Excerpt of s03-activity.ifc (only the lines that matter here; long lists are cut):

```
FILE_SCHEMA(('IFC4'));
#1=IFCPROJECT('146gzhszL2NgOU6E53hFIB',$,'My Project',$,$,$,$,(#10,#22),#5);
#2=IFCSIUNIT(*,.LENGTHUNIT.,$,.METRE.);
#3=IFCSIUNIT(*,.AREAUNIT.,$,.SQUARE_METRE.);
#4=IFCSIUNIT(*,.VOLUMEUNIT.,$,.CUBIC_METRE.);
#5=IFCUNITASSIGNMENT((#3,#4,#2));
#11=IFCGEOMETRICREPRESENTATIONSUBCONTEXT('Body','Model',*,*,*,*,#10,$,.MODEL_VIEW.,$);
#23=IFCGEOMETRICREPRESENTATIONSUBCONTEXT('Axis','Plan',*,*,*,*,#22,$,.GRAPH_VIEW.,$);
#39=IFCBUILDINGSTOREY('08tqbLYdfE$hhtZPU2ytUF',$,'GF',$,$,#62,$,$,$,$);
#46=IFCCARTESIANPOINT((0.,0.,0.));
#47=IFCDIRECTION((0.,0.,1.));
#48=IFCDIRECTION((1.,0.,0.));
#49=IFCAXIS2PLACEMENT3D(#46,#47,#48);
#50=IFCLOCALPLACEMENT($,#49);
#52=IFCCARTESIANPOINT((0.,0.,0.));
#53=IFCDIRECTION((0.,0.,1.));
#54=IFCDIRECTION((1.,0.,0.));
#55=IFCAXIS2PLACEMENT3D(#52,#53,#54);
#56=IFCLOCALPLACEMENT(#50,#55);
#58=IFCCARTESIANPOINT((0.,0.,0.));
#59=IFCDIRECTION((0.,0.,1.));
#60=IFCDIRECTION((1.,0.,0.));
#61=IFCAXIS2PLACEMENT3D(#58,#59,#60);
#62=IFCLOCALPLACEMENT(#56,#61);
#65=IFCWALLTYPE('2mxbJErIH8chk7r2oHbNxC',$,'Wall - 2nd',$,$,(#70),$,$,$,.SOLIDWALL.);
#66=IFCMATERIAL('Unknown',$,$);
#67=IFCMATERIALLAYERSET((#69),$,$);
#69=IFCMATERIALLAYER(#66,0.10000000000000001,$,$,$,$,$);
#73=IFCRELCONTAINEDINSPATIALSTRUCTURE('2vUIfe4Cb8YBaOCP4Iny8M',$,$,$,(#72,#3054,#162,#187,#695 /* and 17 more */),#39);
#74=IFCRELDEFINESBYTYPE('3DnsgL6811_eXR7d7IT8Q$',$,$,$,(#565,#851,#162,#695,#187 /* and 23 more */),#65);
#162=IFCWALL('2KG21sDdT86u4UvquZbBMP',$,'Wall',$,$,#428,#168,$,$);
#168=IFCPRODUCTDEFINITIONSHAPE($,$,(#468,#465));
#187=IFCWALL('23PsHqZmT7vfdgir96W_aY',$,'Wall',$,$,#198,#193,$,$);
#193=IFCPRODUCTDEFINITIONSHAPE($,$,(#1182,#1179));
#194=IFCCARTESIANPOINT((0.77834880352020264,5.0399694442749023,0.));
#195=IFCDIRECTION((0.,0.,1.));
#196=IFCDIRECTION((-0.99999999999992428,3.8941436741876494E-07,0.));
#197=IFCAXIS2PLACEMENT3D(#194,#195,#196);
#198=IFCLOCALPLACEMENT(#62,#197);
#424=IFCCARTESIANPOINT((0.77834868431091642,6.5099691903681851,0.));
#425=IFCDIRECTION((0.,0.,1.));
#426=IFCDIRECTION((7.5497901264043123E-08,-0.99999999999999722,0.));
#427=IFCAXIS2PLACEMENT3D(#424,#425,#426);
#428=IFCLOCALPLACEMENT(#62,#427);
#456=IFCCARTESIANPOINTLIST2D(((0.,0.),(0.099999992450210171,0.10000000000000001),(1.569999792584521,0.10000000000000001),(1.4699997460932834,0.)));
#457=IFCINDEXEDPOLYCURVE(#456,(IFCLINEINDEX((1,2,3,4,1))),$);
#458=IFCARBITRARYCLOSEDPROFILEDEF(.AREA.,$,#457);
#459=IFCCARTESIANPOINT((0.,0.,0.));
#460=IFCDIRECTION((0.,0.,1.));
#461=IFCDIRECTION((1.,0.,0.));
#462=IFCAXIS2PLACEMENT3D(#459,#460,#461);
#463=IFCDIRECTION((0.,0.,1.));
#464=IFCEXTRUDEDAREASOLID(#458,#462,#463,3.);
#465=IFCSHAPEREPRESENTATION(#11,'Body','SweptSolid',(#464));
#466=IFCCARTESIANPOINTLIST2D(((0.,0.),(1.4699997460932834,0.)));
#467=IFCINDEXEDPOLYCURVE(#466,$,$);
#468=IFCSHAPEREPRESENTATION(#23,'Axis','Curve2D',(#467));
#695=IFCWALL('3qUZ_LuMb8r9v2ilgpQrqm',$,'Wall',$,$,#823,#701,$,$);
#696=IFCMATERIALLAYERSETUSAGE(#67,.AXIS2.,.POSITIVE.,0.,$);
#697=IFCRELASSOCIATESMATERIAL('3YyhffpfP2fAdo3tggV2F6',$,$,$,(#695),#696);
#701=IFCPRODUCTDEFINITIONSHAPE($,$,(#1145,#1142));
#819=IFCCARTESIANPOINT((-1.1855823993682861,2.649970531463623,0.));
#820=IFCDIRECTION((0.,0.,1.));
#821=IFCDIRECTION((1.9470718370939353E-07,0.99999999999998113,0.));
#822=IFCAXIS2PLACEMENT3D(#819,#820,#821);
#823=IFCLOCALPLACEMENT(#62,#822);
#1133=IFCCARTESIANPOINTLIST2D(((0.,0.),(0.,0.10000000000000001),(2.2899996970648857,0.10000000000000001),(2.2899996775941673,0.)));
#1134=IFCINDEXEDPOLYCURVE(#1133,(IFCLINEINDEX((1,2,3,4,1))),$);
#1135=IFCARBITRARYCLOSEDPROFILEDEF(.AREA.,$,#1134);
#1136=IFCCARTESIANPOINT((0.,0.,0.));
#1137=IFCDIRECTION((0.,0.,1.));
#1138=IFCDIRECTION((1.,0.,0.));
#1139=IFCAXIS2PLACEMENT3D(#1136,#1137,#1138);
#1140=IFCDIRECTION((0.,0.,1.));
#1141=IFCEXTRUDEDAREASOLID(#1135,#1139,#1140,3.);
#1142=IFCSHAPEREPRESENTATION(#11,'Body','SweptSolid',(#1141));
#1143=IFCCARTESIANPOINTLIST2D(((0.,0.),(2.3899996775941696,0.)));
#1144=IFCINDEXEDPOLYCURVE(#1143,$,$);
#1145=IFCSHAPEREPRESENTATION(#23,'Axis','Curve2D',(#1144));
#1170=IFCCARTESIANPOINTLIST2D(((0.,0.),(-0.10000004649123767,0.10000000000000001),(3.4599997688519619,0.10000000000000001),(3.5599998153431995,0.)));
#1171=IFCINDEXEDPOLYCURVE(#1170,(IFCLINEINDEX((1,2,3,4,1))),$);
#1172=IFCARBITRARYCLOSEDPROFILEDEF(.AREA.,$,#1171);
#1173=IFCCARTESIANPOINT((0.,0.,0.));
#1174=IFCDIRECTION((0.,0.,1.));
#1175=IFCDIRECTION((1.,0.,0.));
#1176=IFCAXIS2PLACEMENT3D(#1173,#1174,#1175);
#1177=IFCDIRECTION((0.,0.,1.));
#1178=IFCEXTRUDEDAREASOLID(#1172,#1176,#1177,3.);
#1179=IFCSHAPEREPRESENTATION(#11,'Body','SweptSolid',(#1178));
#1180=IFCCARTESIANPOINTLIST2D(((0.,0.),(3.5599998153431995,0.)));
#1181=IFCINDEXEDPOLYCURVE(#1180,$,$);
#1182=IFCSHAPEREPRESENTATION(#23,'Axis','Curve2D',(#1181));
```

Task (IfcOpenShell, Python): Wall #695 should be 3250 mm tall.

```python
import ifcopenshell
import ifcopenshell.geom
import ifcopenshell.util.representation
import ifcopenshell.util.shape
import ifcopenshell.util.unit

model = ifcopenshell.open("s03-activity.ifc")
unit_scale = ifcopenshell.util.unit.calculate_unit_scale(model)
settings = ifcopenshell.geom.settings()


def volume(element):
    """Net volume in cubic metres, openings subtracted."""
    shape = ifcopenshell.geom.create_shape(settings, element)
    return ifcopenshell.util.shape.get_volume(shape.geometry)


wall = model.by_guid("3qUZ_LuMb8r9v2ilgpQrqm")
before = volume(wall)

body = ifcopenshell.util.representation.get_representation(wall, "Model", "Body")
solid = body.Items[0]
old_height = solid.Depth
solid.Depth = 3.25 / unit_scale
after = volume(wall)

print(f"height {old_height:g} -> {solid.Depth:g}, volume {before:.3f} -> {after:.3f} m3")

model.write("s03-activity_rev.ifc")
```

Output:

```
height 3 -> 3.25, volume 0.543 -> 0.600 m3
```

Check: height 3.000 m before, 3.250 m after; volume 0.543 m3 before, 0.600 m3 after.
